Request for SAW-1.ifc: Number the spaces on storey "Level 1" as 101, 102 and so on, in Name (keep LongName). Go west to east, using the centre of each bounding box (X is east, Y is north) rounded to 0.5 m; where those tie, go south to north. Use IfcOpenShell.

First a look at what the model holds.

```python
import ifcopenshell
import ifcopenshell.util.element
import ifcopenshell.util.placement

model = ifcopenshell.open("SAW-1.ifc")
print(model.schema)
storey = next(s for s in model.by_type("IfcBuildingStorey") if s.Name == "Level 1")
spaces = [e for e in ifcopenshell.util.element.get_decomposition(storey) if e.is_a("IfcSpace")]
for e in sorted(spaces, key=lambda e: e.id()):
    origin = ifcopenshell.util.placement.get_local_placement(e.ObjectPlacement)[:3, 3]
    print(e.id(), e.Name, e.LongName, origin.round(2) + 0.0, sep=" | ")
```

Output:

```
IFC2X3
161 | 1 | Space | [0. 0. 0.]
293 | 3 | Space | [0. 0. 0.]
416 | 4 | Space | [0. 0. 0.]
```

```python
import ifcopenshell
import ifcopenshell.geom
import ifcopenshell.util.element
import ifcopenshell.util.shape

model = ifcopenshell.open("SAW-1.ifc")
settings = ifcopenshell.geom.settings()
settings.set("use-world-coords", True)


def centre(element):
    shape = ifcopenshell.geom.create_shape(settings, element)
    return ifcopenshell.util.shape.get_bbox_centroid(shape.geometry)


storey = next(s for s in model.by_type("IfcBuildingStorey") if s.Name == "Level 1")
spaces = [e for e in ifcopenshell.util.element.get_decomposition(storey) if e.is_a("IfcSpace")]

# Insertion points can sit at a corner or the storey origin, so sort by the geometry (in metres).
centres = {e: centre(e) for e in spaces}
spaces.sort(key=lambda e: (round(centres[e][0] / 0.5), centres[e][1]))

for i, e in enumerate(spaces, start=1):
    number = f"1{i:02d}"
    e.Name = number
    print(e.id(), number)

model.write("SAW-1_v2.ifc")
```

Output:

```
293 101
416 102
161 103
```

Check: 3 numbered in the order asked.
